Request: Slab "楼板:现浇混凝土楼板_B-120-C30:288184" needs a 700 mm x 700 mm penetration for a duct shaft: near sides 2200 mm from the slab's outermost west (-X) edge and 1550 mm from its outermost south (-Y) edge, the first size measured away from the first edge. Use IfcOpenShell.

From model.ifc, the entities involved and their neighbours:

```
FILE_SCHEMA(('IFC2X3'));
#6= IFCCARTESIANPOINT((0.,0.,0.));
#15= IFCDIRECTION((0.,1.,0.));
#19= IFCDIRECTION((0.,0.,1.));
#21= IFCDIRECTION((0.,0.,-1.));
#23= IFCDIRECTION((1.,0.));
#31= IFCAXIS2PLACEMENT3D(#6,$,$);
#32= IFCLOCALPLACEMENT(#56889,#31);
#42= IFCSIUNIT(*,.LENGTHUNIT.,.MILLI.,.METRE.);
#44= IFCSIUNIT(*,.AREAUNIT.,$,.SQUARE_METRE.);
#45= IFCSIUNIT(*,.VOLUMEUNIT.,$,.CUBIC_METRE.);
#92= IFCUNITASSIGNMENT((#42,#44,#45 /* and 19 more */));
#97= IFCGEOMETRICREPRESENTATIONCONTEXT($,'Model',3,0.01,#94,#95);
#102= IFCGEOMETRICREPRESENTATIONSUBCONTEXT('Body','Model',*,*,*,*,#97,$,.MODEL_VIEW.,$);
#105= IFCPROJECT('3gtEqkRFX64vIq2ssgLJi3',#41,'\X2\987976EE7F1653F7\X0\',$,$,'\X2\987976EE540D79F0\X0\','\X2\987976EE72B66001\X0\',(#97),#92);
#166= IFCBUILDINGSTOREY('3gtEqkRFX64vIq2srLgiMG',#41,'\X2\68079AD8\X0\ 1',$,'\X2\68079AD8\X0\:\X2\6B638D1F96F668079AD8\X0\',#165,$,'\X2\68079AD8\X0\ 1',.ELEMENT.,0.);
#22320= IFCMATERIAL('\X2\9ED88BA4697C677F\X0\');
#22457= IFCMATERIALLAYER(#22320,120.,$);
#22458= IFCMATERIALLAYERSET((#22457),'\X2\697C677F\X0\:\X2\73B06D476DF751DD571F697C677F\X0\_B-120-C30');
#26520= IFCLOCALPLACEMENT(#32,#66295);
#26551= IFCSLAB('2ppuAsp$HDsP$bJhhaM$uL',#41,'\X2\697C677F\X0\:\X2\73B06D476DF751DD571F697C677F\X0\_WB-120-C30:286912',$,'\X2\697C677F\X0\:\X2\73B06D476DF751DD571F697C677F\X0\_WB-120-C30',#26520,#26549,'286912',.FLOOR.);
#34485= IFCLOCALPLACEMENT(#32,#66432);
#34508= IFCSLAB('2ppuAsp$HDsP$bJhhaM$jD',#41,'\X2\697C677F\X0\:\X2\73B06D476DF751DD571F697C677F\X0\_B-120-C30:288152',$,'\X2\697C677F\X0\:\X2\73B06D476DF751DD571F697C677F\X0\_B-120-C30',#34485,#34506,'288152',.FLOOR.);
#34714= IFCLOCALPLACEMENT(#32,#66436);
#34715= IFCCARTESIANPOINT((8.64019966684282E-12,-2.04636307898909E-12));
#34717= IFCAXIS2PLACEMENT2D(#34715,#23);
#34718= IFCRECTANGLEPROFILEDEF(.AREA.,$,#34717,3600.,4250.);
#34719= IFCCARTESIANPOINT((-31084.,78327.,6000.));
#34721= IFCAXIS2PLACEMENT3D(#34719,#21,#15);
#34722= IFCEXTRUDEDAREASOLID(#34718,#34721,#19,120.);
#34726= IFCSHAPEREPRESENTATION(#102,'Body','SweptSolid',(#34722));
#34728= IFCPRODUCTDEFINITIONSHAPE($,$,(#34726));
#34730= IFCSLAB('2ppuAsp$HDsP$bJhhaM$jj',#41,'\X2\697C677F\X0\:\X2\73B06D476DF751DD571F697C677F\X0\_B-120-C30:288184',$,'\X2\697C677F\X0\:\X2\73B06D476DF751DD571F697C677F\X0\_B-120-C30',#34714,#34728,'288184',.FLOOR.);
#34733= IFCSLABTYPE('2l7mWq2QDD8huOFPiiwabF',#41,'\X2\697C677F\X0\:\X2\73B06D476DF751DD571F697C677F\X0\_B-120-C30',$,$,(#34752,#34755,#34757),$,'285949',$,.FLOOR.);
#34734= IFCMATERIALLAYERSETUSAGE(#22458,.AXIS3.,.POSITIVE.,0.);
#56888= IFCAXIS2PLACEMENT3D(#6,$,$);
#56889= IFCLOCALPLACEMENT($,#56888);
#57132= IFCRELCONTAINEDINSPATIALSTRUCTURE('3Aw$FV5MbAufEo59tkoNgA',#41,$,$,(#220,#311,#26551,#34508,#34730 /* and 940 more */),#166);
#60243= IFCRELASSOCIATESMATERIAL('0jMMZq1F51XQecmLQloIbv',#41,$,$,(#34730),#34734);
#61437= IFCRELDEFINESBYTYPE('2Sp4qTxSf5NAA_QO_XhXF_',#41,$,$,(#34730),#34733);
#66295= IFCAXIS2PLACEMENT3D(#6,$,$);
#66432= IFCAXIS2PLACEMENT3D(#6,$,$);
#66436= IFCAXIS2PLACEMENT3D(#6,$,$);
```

```python
import numpy as np
import ifcopenshell
import ifcopenshell.api.feature
import ifcopenshell.api.geometry
import ifcopenshell.api.root
import ifcopenshell.geom
import ifcopenshell.util.placement
import ifcopenshell.util.representation
import ifcopenshell.util.shape
import ifcopenshell.util.unit

model = ifcopenshell.open("model.ifc")
unit_scale = ifcopenshell.util.unit.calculate_unit_scale(model)
settings = ifcopenshell.geom.settings()


def volume(element):
    """Net volume in cubic metres, openings subtracted."""
    shape = ifcopenshell.geom.create_shape(settings, element)
    return ifcopenshell.util.shape.get_volume(shape.geometry)


slab = model.by_id(34730)
before = volume(slab)

# Extent in the slab's own axes, in metres. The edges named are its -X and -Y sides.
slab_shape = ifcopenshell.geom.create_shape(settings, slab)
vertices = ifcopenshell.util.shape.get_vertices(slab_shape.geometry)
x_min, y_min, bottom = vertices.min(axis=0)
top = vertices[:, 2].max()

opening = ifcopenshell.api.root.create_entity(model, ifc_class="IfcOpeningElement", name="Duct shaft opening")
context = ifcopenshell.util.representation.get_context(model, "Model", "Body", "MODEL_VIEW")
width, depth = 0.7, 0.7
outline = [(0.0, 0.0), (width, 0.0), (width, depth), (0.0, depth), (0.0, 0.0)]
# Overshoot both faces by 50 mm so the cut is clean.
shape = ifcopenshell.api.geometry.add_slab_representation(
    model, context=context, depth=top - bottom + 0.1, polyline=outline
)
ifcopenshell.api.geometry.assign_representation(model, product=opening, representation=shape)

matrix = ifcopenshell.util.placement.get_local_placement(slab.ObjectPlacement)
matrix[:, 3] = matrix @ np.append(np.array([x_min + 2.2, y_min + 1.55, bottom - 0.05]) / unit_scale, 1.0)
ifcopenshell.api.geometry.edit_object_placement(model, product=opening, matrix=matrix, is_si=False)
ifcopenshell.api.feature.add_feature(model, feature=opening, element=slab)

after = volume(slab)

print(f"slab volume {before:.3f} -> {after:.3f} m3")

model.write("model_edited.ifc")
```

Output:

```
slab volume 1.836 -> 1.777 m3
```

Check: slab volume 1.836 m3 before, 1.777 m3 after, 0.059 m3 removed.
